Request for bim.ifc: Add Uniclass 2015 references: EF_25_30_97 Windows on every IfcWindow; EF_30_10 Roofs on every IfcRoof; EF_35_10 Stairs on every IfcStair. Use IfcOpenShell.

First a look at what the model holds.

```python
import ifcopenshell

model = ifcopenshell.open("bim.ifc")
print(model.schema)
print("classifications:", [c.Name for c in model.by_type("IfcClassification")])
for ifc_class in ("IfcDoor", "IfcRoof", "IfcStair", "IfcWall", "IfcWindow"):
    print(ifc_class, len(model.by_type(ifc_class)))
```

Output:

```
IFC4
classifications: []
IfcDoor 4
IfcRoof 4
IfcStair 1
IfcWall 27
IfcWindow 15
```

```python
import ifcopenshell
import ifcopenshell.api.classification

model = ifcopenshell.open("bim.ifc")

system = ifcopenshell.api.classification.add_classification(model, classification="Uniclass 2015")

codes = {
    "IfcWindow": ("EF_25_30_97", "Windows"),
    "IfcRoof": ("EF_30_10", "Roofs"),
    "IfcStair": ("EF_35_10", "Stairs"),
}
for ifc_class, (code, name) in codes.items():
    products = model.by_type(ifc_class)
    ifcopenshell.api.classification.add_reference(
        model, products=products, classification=system, identification=code, name=name
    )
    print(code, len(products))

model.write("bim_v2.ifc")
```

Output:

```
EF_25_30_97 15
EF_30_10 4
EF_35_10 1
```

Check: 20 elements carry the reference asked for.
